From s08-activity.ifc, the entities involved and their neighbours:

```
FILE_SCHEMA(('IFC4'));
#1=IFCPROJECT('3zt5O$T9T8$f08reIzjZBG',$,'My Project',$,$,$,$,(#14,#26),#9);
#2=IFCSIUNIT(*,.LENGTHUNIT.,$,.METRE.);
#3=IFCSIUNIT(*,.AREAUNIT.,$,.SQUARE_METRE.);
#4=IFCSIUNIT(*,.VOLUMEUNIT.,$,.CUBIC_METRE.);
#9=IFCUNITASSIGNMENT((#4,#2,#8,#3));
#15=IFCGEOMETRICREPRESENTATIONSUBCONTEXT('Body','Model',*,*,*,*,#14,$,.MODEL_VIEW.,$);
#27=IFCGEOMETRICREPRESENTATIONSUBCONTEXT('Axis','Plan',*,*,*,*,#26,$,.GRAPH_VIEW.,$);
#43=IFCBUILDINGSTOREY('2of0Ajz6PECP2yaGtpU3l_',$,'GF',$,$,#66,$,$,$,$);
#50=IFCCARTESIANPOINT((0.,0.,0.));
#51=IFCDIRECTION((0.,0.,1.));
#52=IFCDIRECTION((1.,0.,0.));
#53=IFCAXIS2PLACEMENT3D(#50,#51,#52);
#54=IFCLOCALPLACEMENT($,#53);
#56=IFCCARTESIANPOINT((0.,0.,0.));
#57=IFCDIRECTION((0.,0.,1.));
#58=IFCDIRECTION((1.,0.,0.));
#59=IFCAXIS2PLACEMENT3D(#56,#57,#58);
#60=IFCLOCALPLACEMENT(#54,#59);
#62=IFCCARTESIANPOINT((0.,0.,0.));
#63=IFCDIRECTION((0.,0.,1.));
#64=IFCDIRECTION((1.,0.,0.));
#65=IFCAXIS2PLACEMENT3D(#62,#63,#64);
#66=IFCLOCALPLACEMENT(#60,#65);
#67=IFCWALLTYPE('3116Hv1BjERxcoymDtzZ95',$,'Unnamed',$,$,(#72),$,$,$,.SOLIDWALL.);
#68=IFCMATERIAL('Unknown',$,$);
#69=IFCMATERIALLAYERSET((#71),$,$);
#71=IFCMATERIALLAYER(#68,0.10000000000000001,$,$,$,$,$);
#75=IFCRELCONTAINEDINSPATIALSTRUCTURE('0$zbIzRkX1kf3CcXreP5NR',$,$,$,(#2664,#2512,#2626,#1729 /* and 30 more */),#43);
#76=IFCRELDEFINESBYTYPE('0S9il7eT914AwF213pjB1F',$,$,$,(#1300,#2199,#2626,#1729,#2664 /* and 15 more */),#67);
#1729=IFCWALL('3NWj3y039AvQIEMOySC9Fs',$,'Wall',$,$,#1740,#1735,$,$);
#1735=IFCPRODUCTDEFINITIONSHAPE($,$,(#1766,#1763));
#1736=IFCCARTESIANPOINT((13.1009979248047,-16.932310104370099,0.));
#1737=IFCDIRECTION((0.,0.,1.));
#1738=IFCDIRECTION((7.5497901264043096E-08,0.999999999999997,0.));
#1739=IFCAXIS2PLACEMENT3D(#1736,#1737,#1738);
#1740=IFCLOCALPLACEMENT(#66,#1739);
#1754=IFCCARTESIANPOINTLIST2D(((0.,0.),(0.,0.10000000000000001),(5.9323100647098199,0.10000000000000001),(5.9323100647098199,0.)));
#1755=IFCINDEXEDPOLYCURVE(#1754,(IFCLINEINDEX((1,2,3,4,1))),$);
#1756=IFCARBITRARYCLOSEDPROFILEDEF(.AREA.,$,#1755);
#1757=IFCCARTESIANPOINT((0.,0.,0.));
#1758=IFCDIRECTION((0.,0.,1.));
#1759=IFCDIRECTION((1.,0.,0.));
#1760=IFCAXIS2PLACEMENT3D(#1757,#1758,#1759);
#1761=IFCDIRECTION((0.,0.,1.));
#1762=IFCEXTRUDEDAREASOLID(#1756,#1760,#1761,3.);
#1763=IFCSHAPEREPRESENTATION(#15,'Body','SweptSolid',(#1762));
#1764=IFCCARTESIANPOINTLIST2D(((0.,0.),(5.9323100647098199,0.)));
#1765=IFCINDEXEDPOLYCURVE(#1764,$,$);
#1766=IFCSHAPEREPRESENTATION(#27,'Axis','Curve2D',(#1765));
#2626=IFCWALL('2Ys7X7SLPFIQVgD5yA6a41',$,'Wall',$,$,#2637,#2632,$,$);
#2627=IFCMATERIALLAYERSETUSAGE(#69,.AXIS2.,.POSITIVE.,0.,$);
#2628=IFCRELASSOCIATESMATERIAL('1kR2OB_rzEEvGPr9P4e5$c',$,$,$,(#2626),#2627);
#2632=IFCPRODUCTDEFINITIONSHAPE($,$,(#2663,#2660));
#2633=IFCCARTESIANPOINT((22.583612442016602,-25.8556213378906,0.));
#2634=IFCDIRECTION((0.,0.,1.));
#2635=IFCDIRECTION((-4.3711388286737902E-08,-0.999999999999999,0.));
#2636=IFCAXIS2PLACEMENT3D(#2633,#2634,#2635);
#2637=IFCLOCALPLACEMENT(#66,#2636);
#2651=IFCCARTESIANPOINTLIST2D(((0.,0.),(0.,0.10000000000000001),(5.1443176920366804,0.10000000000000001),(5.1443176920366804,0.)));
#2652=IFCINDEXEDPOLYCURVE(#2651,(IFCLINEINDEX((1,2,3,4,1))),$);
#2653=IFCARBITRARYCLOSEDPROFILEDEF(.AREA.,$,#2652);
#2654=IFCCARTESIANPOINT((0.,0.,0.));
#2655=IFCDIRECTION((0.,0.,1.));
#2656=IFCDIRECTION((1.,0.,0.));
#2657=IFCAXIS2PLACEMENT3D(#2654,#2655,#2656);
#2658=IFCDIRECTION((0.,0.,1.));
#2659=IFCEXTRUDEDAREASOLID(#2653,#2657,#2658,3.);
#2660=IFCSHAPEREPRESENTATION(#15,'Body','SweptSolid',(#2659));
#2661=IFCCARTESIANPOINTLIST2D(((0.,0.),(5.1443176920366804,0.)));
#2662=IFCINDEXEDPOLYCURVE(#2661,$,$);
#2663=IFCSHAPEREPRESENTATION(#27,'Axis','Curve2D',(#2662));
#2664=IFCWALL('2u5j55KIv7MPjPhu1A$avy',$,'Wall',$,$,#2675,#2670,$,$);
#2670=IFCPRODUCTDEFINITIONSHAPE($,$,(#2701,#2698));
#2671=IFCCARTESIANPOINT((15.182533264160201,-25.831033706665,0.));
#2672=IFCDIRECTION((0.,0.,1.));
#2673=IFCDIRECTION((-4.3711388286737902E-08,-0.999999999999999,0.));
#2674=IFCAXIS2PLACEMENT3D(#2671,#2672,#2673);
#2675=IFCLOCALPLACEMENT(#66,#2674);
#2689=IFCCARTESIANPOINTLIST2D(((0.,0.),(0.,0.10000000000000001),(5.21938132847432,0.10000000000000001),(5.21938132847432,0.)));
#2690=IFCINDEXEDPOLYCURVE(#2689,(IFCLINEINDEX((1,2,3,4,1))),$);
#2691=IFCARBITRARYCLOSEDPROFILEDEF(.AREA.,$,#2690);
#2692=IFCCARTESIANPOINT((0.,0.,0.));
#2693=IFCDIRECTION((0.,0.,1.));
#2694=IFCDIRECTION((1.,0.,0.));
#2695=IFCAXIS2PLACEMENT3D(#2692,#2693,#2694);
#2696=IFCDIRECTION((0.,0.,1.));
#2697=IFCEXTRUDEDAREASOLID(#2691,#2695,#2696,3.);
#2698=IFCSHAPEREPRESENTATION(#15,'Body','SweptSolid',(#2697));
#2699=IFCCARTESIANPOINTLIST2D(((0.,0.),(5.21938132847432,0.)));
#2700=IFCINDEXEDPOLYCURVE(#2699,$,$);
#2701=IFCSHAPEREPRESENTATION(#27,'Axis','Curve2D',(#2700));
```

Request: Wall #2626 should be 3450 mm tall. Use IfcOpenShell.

```python
import ifcopenshell
import ifcopenshell.geom
import ifcopenshell.util.representation
import ifcopenshell.util.shape

model = ifcopenshell.open("s08-activity.ifc")
settings = ifcopenshell.geom.settings()


def volume(element):
    """Net volume in cubic metres, openings subtracted."""
    shape = ifcopenshell.geom.create_shape(settings, element)
    return ifcopenshell.util.shape.get_volume(shape.geometry)


wall = model.by_id(2626)
before = volume(wall)

body = ifcopenshell.util.representation.get_representation(wall, "Model", "Body")
solid = body.Items[0]
old_height = solid.Depth
solid.Depth = 3.45
after = volume(wall)

print(f"height {old_height:g} -> {solid.Depth:g}, volume {before:.3f} -> {after:.3f} m3")

model.write("s08-activity_edited.ifc")
```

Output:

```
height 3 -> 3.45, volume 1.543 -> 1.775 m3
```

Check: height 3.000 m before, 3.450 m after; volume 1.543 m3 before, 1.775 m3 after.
